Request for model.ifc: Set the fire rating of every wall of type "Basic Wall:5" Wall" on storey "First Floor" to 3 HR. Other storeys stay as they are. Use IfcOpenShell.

First a look at what the model holds.

```python
import ifcopenshell
import ifcopenshell.util.element

model = ifcopenshell.open("model.ifc")
print(model.schema)
storey = next(s for s in model.by_type("IfcBuildingStorey") if s.Name == "First Floor")
walls = [e for e in ifcopenshell.util.element.get_decomposition(storey) if e.is_a("IfcWall")]
seen = {}
for e in walls:
    element_type = ifcopenshell.util.element.get_type(e)
    key = (element_type.Name if element_type != e and element_type else None, ifcopenshell.util.element.get_pset(e, "Pset_WallCommon", "FireRating"))
    seen[key] = seen.get(key, 0) + 1
for (name, value), count in sorted(seen.items(), key=str):
    print(count, "x", name, "|", value)
```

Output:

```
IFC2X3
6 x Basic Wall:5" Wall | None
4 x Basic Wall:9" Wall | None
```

```python
import ifcopenshell
import ifcopenshell.api.pset
import ifcopenshell.util.element

model = ifcopenshell.open("model.ifc")

storey = next(s for s in model.by_type("IfcBuildingStorey") if s.Name == "First Floor")
walls = [e for e in ifcopenshell.util.element.get_decomposition(storey) if e.is_a("IfcWall")]

count = 0
for e in walls:
    element_type = ifcopenshell.util.element.get_type(e)
    if element_type in (None, e) or element_type.Name != 'Basic Wall:5" Wall':
        continue
    # add_pset returns the element's existing set when there is one.
    pset = ifcopenshell.api.pset.add_pset(model, product=e, name="Pset_WallCommon")
    ifcopenshell.api.pset.edit_pset(model, pset=pset, properties={"FireRating": "3 HR"})
    count += 1

print(count, "walls updated")

model.write("model_rev.ifc")
```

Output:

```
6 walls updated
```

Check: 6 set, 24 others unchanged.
